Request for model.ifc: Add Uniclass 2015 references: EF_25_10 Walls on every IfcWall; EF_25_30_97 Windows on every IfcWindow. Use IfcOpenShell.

First a look at what the model holds.

```python
import ifcopenshell

model = ifcopenshell.open("model.ifc")
print(model.schema)
print("classifications:", [c.Name for c in model.by_type("IfcClassification")])
for ifc_class in ("IfcDoor", "IfcRoof", "IfcStair", "IfcWall", "IfcWindow"):
    print(ifc_class, len(model.by_type(ifc_class)))
```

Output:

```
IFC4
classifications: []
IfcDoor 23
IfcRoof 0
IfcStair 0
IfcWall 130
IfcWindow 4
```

```python
import ifcopenshell
import ifcopenshell.api.classification

model = ifcopenshell.open("model.ifc")

system = ifcopenshell.api.classification.add_classification(model, classification="Uniclass 2015")

codes = {
    "IfcWall": ("EF_25_10", "Walls"),
    "IfcWindow": ("EF_25_30_97", "Windows"),
}
for ifc_class, (code, name) in codes.items():
    products = model.by_type(ifc_class)
    ifcopenshell.api.classification.add_reference(
        model, products=products, classification=system, identification=code, name=name
    )
    print(code, len(products))

model.write("model_v2.ifc")
```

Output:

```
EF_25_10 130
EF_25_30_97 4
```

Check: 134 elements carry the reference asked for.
